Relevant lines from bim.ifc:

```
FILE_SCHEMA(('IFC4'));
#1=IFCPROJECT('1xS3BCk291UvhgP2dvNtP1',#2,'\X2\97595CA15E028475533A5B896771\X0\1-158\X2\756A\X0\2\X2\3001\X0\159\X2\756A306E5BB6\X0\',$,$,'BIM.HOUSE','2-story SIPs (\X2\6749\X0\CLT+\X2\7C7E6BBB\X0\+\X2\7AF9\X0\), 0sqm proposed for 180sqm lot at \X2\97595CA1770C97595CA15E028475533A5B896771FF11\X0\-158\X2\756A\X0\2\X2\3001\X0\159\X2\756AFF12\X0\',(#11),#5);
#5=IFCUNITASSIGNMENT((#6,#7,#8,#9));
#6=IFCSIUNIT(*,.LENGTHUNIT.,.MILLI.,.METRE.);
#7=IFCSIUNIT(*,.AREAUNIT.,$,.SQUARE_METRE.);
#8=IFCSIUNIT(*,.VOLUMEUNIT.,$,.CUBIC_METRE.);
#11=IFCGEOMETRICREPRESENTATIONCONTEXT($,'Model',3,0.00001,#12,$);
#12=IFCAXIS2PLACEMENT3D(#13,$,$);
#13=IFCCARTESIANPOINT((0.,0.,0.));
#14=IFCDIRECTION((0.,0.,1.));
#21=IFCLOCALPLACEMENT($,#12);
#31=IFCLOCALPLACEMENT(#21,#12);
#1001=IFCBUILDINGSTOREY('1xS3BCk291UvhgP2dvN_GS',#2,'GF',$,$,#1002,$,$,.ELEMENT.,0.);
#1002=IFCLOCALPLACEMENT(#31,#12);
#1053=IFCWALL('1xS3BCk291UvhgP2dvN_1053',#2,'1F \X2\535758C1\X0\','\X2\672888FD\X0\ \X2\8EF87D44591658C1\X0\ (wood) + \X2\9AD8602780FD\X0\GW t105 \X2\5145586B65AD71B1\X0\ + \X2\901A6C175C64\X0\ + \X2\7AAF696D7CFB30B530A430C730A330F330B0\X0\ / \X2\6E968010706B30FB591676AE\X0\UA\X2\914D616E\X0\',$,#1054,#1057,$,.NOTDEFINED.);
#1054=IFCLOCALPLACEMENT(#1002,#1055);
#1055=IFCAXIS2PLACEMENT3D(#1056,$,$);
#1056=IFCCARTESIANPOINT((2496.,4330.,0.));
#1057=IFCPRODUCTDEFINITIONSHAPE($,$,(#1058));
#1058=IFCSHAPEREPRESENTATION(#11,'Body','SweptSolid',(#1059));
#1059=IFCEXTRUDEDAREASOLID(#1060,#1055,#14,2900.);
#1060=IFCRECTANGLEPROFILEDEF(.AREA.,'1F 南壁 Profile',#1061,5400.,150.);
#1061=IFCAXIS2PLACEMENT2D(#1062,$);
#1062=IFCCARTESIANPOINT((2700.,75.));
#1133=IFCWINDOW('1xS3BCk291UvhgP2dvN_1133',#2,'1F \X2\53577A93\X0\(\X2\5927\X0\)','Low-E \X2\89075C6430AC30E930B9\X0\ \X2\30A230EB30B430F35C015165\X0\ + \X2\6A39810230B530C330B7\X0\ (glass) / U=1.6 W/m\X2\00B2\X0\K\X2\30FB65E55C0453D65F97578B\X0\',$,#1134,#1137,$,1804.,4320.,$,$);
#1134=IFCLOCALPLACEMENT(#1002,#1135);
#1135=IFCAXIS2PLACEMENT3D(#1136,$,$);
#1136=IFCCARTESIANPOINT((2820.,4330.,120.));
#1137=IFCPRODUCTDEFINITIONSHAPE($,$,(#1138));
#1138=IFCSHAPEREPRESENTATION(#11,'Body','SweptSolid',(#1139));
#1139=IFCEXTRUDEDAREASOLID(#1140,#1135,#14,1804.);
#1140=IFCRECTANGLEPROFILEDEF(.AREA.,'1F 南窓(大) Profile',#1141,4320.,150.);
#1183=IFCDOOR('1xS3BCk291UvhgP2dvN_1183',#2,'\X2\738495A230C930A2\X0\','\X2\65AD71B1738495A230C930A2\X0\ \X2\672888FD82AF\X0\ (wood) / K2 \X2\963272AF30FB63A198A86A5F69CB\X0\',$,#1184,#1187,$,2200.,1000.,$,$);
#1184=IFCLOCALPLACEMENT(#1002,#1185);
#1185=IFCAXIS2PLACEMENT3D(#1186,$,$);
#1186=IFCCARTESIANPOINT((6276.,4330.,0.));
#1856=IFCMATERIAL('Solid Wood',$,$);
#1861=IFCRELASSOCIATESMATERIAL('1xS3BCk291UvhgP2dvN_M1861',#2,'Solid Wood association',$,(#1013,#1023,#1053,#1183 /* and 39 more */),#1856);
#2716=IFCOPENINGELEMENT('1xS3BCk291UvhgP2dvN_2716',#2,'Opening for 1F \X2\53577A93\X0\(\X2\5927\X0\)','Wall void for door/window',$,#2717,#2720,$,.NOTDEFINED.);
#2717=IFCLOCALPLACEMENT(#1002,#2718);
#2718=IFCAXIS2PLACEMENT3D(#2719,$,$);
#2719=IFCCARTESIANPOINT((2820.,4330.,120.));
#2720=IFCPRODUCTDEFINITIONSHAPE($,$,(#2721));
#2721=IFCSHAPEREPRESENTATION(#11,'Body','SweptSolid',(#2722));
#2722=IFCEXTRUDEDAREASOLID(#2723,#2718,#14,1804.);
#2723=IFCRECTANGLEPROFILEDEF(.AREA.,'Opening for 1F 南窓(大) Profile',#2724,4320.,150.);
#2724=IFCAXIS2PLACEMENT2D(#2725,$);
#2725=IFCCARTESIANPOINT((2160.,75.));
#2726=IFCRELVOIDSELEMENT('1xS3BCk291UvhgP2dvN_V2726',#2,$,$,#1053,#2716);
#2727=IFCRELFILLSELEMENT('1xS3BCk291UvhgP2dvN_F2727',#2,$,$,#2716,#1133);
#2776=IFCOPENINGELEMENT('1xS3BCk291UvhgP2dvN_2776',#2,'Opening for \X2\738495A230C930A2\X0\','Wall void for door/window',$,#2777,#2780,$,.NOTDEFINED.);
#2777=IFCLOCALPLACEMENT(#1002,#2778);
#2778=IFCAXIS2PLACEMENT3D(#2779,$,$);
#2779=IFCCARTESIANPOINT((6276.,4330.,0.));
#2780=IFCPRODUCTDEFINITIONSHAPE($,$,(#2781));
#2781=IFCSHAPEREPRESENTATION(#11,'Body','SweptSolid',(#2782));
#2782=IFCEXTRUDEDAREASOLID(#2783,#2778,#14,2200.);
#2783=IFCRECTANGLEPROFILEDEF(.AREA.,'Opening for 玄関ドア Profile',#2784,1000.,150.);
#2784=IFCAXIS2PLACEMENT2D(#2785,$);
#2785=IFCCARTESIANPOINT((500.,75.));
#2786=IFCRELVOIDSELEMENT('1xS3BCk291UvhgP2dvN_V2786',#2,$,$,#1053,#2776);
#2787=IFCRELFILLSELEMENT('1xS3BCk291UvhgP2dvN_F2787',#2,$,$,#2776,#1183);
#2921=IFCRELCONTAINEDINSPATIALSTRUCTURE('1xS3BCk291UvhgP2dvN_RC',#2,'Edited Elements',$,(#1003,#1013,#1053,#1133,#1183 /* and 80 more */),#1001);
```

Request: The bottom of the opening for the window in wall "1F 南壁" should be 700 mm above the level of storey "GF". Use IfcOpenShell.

```python
import numpy as np
import ifcopenshell
import ifcopenshell.api.geometry
import ifcopenshell.geom
import ifcopenshell.util.element
import ifcopenshell.util.placement
import ifcopenshell.util.shape
import ifcopenshell.util.unit

model = ifcopenshell.open("bim.ifc")
unit_scale = ifcopenshell.util.unit.calculate_unit_scale(model)

window = model.by_id(1133)
opening = window.FillsVoids[0].RelatingOpeningElement
storey = ifcopenshell.util.element.get_container(window, ifc_class="IfcBuildingStorey")
level = ifcopenshell.util.placement.get_local_placement(storey.ObjectPlacement)[2, 3]

# The opening's origin need not be at the sill, so measure its lowest point.
shape = ifcopenshell.geom.create_shape(ifcopenshell.geom.settings(), opening)
bottom = ifcopenshell.util.shape.get_shape_bottom_elevation(shape, shape.geometry) / unit_scale
dz = level + 0.7 / unit_scale - bottom

shift = np.array([0.0, 0.0, dz])
# The window is not placed relative to its opening, so move both.
for product in (opening, window):
    matrix = ifcopenshell.util.placement.get_local_placement(product.ObjectPlacement)
    matrix[:3, 3] += shift
    ifcopenshell.api.geometry.edit_object_placement(model, product=product, matrix=matrix, is_si=False)

print(f"moved by {dz * unit_scale:+.3f} m")

model.write("bim-out.ifc")
```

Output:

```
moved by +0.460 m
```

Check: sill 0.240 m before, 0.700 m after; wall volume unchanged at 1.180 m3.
